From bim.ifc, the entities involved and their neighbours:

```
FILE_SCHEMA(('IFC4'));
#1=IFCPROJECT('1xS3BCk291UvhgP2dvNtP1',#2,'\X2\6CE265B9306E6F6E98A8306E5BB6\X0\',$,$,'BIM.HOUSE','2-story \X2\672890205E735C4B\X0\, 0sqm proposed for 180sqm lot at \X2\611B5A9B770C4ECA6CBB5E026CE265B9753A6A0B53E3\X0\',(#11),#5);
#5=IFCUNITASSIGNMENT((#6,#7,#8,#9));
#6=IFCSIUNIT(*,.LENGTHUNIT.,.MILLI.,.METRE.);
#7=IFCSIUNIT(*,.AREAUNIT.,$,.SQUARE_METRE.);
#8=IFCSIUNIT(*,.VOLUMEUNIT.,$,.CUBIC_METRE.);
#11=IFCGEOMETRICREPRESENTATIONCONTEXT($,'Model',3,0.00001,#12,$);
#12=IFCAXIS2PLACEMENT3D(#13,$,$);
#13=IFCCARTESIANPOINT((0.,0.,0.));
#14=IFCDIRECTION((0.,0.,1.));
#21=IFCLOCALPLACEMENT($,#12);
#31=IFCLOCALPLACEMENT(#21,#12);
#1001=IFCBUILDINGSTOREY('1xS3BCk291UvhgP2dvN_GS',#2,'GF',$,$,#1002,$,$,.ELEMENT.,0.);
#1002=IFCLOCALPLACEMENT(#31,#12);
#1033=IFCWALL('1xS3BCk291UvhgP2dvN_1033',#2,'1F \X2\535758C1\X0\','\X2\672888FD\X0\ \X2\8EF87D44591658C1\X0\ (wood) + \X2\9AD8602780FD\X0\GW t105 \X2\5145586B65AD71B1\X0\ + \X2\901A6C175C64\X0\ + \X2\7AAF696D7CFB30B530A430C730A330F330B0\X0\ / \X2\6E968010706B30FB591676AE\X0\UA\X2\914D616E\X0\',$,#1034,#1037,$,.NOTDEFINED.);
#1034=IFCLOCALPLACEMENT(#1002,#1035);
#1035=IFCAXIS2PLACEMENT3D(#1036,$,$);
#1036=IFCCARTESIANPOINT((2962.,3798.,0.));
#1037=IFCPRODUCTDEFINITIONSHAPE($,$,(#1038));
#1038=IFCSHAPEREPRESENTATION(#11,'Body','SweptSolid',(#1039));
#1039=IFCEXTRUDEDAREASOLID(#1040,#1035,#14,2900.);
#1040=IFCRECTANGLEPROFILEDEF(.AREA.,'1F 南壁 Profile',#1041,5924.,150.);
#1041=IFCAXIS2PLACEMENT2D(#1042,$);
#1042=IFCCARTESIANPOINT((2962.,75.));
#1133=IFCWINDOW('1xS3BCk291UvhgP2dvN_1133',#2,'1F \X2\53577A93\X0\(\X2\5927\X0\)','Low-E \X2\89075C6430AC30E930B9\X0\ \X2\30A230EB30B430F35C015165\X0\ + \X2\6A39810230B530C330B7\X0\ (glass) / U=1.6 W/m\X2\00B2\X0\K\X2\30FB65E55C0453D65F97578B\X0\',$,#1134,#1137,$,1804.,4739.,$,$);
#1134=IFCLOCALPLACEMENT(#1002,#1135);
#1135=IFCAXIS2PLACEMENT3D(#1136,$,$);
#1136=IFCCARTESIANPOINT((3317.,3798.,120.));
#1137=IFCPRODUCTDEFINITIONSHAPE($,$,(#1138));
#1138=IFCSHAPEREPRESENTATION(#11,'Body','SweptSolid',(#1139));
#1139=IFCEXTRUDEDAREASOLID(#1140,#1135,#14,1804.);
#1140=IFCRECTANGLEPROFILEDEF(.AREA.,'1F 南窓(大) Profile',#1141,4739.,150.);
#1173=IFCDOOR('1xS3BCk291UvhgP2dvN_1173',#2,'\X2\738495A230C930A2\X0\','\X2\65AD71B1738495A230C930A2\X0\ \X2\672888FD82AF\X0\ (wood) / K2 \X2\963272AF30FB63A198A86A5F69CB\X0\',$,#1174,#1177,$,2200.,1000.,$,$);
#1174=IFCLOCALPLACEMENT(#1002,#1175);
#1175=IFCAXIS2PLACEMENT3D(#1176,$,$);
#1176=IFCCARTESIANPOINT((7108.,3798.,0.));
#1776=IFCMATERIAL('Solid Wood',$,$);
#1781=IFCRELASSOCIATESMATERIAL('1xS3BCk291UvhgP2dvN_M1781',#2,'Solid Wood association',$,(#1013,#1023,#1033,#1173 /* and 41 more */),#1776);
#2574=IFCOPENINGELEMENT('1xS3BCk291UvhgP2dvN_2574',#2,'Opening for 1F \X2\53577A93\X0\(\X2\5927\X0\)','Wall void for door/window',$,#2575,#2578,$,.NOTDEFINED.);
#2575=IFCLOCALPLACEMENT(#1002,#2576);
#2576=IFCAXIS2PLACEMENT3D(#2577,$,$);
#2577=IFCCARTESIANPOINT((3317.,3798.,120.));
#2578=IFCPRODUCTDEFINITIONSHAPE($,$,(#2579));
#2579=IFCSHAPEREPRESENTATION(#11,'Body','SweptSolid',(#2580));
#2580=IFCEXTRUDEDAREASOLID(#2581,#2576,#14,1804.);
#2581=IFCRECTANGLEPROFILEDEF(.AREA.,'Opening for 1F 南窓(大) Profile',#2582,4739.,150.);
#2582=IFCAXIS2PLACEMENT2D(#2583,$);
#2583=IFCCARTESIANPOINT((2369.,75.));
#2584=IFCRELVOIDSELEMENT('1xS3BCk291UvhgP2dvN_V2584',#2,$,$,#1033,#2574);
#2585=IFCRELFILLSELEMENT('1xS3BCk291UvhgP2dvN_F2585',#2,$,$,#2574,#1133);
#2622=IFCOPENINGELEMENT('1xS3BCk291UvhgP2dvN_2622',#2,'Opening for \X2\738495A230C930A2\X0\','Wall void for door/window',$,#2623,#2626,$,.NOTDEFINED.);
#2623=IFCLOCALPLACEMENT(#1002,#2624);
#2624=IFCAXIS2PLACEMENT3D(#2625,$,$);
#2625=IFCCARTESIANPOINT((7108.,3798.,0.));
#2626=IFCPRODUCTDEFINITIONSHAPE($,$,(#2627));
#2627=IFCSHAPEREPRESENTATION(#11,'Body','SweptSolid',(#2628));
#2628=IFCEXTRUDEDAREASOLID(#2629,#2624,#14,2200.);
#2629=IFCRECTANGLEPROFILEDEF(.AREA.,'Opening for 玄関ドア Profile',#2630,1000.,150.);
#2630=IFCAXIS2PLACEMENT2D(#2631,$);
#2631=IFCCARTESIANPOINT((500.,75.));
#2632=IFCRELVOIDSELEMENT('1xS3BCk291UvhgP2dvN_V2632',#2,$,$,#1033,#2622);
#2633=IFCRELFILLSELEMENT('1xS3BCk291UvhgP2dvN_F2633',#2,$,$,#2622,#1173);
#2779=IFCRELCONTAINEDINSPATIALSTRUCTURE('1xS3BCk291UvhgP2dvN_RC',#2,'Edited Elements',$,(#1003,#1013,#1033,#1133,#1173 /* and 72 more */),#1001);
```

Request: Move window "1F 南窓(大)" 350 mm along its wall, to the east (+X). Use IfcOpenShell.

```python
import ifcopenshell
import ifcopenshell.api.geometry
import ifcopenshell.util.placement

model = ifcopenshell.open("bim.ifc")

window = model.by_guid("1xS3BCk291UvhgP2dvN_1133")
opening = window.FillsVoids[0].RelatingOpeningElement
wall = opening.VoidsElements[0].RelatingBuildingElement

wall_matrix = ifcopenshell.util.placement.get_local_placement(wall.ObjectPlacement)
shift = wall_matrix[:3, 0] * 350.0
before = ifcopenshell.util.placement.get_local_placement(window.ObjectPlacement)[:3, 3].copy()

# The window is not placed relative to its opening, so move both.
for product in (opening, window):
    matrix = ifcopenshell.util.placement.get_local_placement(product.ObjectPlacement)
    matrix[:3, 3] += shift
    ifcopenshell.api.geometry.edit_object_placement(model, product=product, matrix=matrix, is_si=False)

after = ifcopenshell.util.placement.get_local_placement(window.ObjectPlacement)[:3, 3]
print("window moved by", (after - before).round(3) + 0.0)

model.write("bim_updated.ifc")
```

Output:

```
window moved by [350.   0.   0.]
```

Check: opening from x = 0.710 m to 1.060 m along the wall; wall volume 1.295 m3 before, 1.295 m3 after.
